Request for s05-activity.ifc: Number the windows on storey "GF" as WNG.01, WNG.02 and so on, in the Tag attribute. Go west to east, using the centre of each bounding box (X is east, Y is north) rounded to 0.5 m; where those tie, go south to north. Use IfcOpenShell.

First a look at what the model holds.

```python
import ifcopenshell
import ifcopenshell.util.element
import ifcopenshell.util.placement

model = ifcopenshell.open("s05-activity.ifc")
print(model.schema)
storey = next(s for s in model.by_type("IfcBuildingStorey") if s.Name == "GF")
windows = [e for e in ifcopenshell.util.element.get_decomposition(storey) if e.is_a("IfcWindow")]
for e in sorted(windows, key=lambda e: e.id()):
    origin = ifcopenshell.util.placement.get_local_placement(e.ObjectPlacement)[:3, 3]
    print(e.id(), e.Tag, e.Name, origin.round(2) + 0.0, sep=" | ")
```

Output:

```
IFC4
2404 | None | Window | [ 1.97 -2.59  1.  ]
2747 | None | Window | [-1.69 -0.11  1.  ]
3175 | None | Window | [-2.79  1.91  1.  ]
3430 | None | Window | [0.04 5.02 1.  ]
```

```python
import ifcopenshell
import ifcopenshell.geom
import ifcopenshell.util.element
import ifcopenshell.util.shape

model = ifcopenshell.open("s05-activity.ifc")
settings = ifcopenshell.geom.settings()
settings.set("use-world-coords", True)


def centre(element):
    shape = ifcopenshell.geom.create_shape(settings, element)
    return ifcopenshell.util.shape.get_bbox_centroid(shape.geometry)


storey = next(s for s in model.by_type("IfcBuildingStorey") if s.Name == "GF")
windows = [e for e in ifcopenshell.util.element.get_decomposition(storey) if e.is_a("IfcWindow")]

# Insertion points can sit at a corner or the storey origin, so sort by the geometry (in metres).
centres = {e: centre(e) for e in windows}
windows.sort(key=lambda e: (round(centres[e][0] / 0.5), centres[e][1]))

for i, e in enumerate(windows, start=1):
    number = f"WNG.{i:02d}"
    e.Tag = number
    print(e.id(), number)

model.write("s05-activity-out.ifc")
```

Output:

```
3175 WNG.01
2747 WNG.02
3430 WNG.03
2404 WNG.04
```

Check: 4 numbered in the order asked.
